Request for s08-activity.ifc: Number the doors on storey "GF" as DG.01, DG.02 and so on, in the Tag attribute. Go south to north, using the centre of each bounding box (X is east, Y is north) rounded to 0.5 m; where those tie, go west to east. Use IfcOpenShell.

First a look at what the model holds.

```python
import ifcopenshell
import ifcopenshell.util.element
import ifcopenshell.util.placement

model = ifcopenshell.open("s08-activity.ifc")
print(model.schema)
storey = next(s for s in model.by_type("IfcBuildingStorey") if s.Name == "GF")
doors = [e for e in ifcopenshell.util.element.get_decomposition(storey) if e.is_a("IfcDoor")]
for e in sorted(doors, key=lambda e: e.id()):
    origin = ifcopenshell.util.placement.get_local_placement(e.ObjectPlacement)[:3, 3]
    print(e.id(), e.Tag, e.Name, origin.round(2) + 0.0, sep=" | ")
```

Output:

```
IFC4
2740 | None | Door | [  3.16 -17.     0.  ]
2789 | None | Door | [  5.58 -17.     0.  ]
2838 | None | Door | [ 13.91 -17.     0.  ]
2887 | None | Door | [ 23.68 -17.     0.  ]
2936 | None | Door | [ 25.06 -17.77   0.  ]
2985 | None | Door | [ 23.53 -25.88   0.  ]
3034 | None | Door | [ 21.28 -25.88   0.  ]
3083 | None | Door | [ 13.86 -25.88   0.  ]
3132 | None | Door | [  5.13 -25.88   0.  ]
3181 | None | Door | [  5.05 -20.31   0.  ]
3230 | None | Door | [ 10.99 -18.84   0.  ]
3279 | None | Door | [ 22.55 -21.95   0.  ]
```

```python
import ifcopenshell
import ifcopenshell.geom
import ifcopenshell.util.element
import ifcopenshell.util.shape

model = ifcopenshell.open("s08-activity.ifc")
settings = ifcopenshell.geom.settings()
settings.set("use-world-coords", True)


def centre(element):
    shape = ifcopenshell.geom.create_shape(settings, element)
    return ifcopenshell.util.shape.get_bbox_centroid(shape.geometry)


storey = next(s for s in model.by_type("IfcBuildingStorey") if s.Name == "GF")
doors = [e for e in ifcopenshell.util.element.get_decomposition(storey) if e.is_a("IfcDoor")]

# Insertion points can sit at a corner or the storey origin, so sort by the geometry (in metres).
centres = {e: centre(e) for e in doors}
doors.sort(key=lambda e: (round(centres[e][1] / 0.5), centres[e][0]))

for i, e in enumerate(doors, start=1):
    number = f"DG.{i:02d}"
    e.Tag = number
    print(e.id(), number)

model.write("s08-activity-out.ifc")
```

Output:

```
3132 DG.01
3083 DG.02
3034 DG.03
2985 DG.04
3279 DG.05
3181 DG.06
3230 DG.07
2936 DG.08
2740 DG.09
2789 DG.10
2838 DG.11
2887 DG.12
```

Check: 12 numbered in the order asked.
